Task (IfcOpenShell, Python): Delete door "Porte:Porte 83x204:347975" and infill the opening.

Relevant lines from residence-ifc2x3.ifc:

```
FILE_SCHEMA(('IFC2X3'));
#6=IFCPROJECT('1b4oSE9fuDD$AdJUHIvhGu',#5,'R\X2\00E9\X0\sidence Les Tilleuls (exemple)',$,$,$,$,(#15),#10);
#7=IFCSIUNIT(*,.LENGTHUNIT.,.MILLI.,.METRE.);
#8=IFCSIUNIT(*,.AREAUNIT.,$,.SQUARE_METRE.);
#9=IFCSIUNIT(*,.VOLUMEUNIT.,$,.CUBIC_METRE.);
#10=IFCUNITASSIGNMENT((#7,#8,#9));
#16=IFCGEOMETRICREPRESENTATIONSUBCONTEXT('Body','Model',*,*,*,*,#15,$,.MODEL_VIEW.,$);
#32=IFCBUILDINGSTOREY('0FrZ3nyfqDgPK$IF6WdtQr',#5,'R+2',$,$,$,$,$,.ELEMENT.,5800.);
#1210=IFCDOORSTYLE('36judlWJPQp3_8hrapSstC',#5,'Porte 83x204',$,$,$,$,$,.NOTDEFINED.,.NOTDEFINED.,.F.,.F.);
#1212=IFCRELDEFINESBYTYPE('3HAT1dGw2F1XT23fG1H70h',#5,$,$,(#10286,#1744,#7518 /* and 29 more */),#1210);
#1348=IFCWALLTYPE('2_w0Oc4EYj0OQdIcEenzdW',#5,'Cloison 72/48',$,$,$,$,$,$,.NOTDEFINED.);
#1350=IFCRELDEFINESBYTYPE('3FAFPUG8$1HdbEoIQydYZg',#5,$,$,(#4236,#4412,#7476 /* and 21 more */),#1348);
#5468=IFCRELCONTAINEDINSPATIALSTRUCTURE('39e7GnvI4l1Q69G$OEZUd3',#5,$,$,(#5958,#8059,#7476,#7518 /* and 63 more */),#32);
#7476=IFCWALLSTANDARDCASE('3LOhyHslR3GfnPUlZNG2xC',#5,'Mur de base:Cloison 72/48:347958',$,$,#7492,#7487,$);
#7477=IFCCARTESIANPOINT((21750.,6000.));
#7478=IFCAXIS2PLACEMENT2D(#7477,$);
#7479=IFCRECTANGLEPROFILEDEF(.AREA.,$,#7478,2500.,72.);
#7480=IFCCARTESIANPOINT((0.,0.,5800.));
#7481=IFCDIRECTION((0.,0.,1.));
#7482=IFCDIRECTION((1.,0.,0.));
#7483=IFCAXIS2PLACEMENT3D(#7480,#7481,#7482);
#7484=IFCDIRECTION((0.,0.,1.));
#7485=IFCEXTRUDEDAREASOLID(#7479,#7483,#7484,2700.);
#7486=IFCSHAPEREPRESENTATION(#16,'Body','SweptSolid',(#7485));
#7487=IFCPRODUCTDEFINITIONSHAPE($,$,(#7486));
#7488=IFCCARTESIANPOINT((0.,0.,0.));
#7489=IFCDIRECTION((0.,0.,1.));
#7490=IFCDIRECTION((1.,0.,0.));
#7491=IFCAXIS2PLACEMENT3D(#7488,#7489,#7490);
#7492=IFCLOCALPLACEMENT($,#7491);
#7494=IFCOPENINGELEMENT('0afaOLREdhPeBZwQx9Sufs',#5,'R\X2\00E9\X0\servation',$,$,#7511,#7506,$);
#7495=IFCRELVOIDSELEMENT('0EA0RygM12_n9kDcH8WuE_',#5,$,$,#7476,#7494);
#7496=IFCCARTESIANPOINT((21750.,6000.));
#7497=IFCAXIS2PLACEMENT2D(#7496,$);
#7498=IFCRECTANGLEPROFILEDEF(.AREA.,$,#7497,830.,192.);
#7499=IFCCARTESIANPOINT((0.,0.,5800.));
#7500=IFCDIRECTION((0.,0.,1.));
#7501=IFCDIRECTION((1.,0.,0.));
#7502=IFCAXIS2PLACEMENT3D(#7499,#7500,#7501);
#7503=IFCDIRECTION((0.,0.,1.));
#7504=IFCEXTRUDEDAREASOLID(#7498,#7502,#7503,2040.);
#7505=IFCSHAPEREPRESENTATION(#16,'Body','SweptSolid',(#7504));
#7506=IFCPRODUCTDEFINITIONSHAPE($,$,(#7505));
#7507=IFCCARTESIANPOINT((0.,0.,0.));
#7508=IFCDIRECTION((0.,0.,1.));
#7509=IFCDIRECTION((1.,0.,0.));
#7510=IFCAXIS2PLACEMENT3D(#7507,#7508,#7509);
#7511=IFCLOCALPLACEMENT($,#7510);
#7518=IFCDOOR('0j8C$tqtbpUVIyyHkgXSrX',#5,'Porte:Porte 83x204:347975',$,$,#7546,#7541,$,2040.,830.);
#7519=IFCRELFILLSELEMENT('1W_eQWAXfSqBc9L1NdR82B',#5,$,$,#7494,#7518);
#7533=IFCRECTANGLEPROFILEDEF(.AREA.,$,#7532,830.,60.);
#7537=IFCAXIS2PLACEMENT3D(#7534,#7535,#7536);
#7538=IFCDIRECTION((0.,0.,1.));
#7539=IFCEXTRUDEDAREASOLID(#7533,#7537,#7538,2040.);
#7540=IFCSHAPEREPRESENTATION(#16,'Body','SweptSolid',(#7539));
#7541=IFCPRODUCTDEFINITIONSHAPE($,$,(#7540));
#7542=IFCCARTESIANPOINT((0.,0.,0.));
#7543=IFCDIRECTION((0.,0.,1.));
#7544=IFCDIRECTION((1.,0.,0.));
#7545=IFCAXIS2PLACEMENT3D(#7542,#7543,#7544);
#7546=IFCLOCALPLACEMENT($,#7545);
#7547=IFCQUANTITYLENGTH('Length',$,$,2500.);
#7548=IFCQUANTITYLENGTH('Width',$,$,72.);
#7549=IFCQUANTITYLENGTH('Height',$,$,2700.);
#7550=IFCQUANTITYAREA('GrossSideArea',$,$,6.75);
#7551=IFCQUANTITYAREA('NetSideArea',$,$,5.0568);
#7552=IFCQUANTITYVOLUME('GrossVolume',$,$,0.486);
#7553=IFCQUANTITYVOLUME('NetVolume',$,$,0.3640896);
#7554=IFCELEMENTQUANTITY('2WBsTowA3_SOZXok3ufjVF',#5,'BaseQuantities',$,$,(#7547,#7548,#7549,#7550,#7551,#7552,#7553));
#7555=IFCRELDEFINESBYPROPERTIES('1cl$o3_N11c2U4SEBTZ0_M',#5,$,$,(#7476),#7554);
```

```python
import ifcopenshell
import ifcopenshell.api.feature
import ifcopenshell.api.pset
import ifcopenshell.api.root
import ifcopenshell.geom
import ifcopenshell.util.element
import ifcopenshell.util.shape
import ifcopenshell.util.unit

model = ifcopenshell.open("residence-ifc2x3.ifc")
area_scale = ifcopenshell.util.unit.calculate_unit_scale(model, "AREAUNIT")
volume_scale = ifcopenshell.util.unit.calculate_unit_scale(model, "VOLUMEUNIT")
settings = ifcopenshell.geom.settings()


def volume(element):
    """Net volume in cubic metres, openings subtracted."""
    shape = ifcopenshell.geom.create_shape(settings, element)
    return ifcopenshell.util.shape.get_volume(shape.geometry)


door = model.by_guid("0j8C$tqtbpUVIyyHkgXSrX")
opening = door.FillsVoids[0].RelatingOpeningElement
wall = opening.VoidsElements[0].RelatingBuildingElement
before = volume(wall)

ifcopenshell.api.root.remove_product(model, product=door)
ifcopenshell.api.feature.remove_feature(model, feature=opening)

after = volume(wall)
thickness = 0.072  # wall thickness in metres

# Update the wall's stored quantities.
qto = model.by_id(ifcopenshell.util.element.get_pset(wall, "BaseQuantities", should_inherit=False)["id"])
ifcopenshell.api.pset.edit_qto(model, qto=qto, properties={
    "NetSideArea": after / thickness / area_scale,
    "NetVolume": after / volume_scale,
})

print(f"wall volume {before:.3f} -> {after:.3f} m3")

model.write("residence-ifc2x3_updated.ifc")
```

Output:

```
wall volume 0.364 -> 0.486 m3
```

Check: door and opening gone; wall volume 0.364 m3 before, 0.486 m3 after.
